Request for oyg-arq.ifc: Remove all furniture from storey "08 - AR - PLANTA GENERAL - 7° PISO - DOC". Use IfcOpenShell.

First a look at what the model holds.

```python
import ifcopenshell
import ifcopenshell.util.element

model = ifcopenshell.open("oyg-arq.ifc")
print(model.schema)
storey = next(s for s in model.by_type("IfcBuildingStorey") if s.Name == "08 - AR - PLANTA GENERAL - 7° PISO - DOC")
furniture = [e for e in ifcopenshell.util.element.get_decomposition(storey) if e.is_a("IfcFurnishingElement")]
seen = {}
for e in furniture:
    element_type = ifcopenshell.util.element.get_type(e)
    name = element_type.Name if element_type not in (None, e) else None
    seen[name] = seen.get(name, 0) + 1
for name, count in sorted(seen.items(), key=str):
    print(count, "x", name)
```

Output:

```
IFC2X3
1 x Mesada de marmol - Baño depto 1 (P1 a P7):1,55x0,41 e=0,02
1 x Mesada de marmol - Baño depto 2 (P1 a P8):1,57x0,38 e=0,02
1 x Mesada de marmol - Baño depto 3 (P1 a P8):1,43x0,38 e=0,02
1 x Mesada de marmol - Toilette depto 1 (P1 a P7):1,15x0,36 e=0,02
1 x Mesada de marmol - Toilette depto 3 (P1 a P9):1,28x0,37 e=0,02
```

```python
import ifcopenshell
import ifcopenshell.api.root
import ifcopenshell.util.element

model = ifcopenshell.open("oyg-arq.ifc")

storey = next(s for s in model.by_type("IfcBuildingStorey") if s.Name == "08 - AR - PLANTA GENERAL - 7° PISO - DOC")
furniture = [e for e in ifcopenshell.util.element.get_decomposition(storey) if e.is_a("IfcFurnishingElement")]

for e in furniture:
    ifcopenshell.api.root.remove_product(model, product=e)
print(len(furniture), "removed")

model.write("oyg-arq_edited.ifc")
```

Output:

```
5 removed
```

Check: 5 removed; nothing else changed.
